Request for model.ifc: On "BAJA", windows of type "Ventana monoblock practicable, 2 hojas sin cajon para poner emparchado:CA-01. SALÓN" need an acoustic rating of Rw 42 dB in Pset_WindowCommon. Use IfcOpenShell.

First a look at what the model holds.

```python
import ifcopenshell
import ifcopenshell.util.element

model = ifcopenshell.open("model.ifc")
print(model.schema)
storey = next(s for s in model.by_type("IfcBuildingStorey") if s.Name == "BAJA")
windows = [e for e in ifcopenshell.util.element.get_decomposition(storey) if e.is_a("IfcWindow")]
seen = {}
for e in windows:
    element_type = ifcopenshell.util.element.get_type(e)
    key = (element_type.Name if element_type != e and element_type else None, ifcopenshell.util.element.get_pset(e, "Pset_WindowCommon", "AcousticRating"))
    seen[key] = seen.get(key, 0) + 1
for (name, value), count in sorted(seen.items(), key=str):
    print(count, "x", name, "|", value)
```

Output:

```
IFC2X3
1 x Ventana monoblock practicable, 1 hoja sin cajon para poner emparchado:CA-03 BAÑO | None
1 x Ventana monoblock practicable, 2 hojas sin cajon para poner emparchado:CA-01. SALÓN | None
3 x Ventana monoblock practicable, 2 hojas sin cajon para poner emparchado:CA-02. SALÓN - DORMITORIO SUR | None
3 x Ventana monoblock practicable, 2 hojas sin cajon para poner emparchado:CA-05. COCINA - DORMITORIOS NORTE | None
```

```python
import ifcopenshell
import ifcopenshell.api.pset
import ifcopenshell.util.element

model = ifcopenshell.open("model.ifc")

storey = next(s for s in model.by_type("IfcBuildingStorey") if s.Name == "BAJA")
windows = [e for e in ifcopenshell.util.element.get_decomposition(storey) if e.is_a("IfcWindow")]

count = 0
for e in windows:
    element_type = ifcopenshell.util.element.get_type(e)
    if element_type in (None, e) or element_type.Name != "Ventana monoblock practicable, 2 hojas sin cajon para poner emparchado:CA-01. SALÓN":
        continue
    # add_pset returns the element's existing set when there is one.
    pset = ifcopenshell.api.pset.add_pset(model, product=e, name="Pset_WindowCommon")
    ifcopenshell.api.pset.edit_pset(model, pset=pset, properties={"AcousticRating": "Rw 42 dB"})
    count += 1

print(count, "windows updated")

model.write("model_v2.ifc")
```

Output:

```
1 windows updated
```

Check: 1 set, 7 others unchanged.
